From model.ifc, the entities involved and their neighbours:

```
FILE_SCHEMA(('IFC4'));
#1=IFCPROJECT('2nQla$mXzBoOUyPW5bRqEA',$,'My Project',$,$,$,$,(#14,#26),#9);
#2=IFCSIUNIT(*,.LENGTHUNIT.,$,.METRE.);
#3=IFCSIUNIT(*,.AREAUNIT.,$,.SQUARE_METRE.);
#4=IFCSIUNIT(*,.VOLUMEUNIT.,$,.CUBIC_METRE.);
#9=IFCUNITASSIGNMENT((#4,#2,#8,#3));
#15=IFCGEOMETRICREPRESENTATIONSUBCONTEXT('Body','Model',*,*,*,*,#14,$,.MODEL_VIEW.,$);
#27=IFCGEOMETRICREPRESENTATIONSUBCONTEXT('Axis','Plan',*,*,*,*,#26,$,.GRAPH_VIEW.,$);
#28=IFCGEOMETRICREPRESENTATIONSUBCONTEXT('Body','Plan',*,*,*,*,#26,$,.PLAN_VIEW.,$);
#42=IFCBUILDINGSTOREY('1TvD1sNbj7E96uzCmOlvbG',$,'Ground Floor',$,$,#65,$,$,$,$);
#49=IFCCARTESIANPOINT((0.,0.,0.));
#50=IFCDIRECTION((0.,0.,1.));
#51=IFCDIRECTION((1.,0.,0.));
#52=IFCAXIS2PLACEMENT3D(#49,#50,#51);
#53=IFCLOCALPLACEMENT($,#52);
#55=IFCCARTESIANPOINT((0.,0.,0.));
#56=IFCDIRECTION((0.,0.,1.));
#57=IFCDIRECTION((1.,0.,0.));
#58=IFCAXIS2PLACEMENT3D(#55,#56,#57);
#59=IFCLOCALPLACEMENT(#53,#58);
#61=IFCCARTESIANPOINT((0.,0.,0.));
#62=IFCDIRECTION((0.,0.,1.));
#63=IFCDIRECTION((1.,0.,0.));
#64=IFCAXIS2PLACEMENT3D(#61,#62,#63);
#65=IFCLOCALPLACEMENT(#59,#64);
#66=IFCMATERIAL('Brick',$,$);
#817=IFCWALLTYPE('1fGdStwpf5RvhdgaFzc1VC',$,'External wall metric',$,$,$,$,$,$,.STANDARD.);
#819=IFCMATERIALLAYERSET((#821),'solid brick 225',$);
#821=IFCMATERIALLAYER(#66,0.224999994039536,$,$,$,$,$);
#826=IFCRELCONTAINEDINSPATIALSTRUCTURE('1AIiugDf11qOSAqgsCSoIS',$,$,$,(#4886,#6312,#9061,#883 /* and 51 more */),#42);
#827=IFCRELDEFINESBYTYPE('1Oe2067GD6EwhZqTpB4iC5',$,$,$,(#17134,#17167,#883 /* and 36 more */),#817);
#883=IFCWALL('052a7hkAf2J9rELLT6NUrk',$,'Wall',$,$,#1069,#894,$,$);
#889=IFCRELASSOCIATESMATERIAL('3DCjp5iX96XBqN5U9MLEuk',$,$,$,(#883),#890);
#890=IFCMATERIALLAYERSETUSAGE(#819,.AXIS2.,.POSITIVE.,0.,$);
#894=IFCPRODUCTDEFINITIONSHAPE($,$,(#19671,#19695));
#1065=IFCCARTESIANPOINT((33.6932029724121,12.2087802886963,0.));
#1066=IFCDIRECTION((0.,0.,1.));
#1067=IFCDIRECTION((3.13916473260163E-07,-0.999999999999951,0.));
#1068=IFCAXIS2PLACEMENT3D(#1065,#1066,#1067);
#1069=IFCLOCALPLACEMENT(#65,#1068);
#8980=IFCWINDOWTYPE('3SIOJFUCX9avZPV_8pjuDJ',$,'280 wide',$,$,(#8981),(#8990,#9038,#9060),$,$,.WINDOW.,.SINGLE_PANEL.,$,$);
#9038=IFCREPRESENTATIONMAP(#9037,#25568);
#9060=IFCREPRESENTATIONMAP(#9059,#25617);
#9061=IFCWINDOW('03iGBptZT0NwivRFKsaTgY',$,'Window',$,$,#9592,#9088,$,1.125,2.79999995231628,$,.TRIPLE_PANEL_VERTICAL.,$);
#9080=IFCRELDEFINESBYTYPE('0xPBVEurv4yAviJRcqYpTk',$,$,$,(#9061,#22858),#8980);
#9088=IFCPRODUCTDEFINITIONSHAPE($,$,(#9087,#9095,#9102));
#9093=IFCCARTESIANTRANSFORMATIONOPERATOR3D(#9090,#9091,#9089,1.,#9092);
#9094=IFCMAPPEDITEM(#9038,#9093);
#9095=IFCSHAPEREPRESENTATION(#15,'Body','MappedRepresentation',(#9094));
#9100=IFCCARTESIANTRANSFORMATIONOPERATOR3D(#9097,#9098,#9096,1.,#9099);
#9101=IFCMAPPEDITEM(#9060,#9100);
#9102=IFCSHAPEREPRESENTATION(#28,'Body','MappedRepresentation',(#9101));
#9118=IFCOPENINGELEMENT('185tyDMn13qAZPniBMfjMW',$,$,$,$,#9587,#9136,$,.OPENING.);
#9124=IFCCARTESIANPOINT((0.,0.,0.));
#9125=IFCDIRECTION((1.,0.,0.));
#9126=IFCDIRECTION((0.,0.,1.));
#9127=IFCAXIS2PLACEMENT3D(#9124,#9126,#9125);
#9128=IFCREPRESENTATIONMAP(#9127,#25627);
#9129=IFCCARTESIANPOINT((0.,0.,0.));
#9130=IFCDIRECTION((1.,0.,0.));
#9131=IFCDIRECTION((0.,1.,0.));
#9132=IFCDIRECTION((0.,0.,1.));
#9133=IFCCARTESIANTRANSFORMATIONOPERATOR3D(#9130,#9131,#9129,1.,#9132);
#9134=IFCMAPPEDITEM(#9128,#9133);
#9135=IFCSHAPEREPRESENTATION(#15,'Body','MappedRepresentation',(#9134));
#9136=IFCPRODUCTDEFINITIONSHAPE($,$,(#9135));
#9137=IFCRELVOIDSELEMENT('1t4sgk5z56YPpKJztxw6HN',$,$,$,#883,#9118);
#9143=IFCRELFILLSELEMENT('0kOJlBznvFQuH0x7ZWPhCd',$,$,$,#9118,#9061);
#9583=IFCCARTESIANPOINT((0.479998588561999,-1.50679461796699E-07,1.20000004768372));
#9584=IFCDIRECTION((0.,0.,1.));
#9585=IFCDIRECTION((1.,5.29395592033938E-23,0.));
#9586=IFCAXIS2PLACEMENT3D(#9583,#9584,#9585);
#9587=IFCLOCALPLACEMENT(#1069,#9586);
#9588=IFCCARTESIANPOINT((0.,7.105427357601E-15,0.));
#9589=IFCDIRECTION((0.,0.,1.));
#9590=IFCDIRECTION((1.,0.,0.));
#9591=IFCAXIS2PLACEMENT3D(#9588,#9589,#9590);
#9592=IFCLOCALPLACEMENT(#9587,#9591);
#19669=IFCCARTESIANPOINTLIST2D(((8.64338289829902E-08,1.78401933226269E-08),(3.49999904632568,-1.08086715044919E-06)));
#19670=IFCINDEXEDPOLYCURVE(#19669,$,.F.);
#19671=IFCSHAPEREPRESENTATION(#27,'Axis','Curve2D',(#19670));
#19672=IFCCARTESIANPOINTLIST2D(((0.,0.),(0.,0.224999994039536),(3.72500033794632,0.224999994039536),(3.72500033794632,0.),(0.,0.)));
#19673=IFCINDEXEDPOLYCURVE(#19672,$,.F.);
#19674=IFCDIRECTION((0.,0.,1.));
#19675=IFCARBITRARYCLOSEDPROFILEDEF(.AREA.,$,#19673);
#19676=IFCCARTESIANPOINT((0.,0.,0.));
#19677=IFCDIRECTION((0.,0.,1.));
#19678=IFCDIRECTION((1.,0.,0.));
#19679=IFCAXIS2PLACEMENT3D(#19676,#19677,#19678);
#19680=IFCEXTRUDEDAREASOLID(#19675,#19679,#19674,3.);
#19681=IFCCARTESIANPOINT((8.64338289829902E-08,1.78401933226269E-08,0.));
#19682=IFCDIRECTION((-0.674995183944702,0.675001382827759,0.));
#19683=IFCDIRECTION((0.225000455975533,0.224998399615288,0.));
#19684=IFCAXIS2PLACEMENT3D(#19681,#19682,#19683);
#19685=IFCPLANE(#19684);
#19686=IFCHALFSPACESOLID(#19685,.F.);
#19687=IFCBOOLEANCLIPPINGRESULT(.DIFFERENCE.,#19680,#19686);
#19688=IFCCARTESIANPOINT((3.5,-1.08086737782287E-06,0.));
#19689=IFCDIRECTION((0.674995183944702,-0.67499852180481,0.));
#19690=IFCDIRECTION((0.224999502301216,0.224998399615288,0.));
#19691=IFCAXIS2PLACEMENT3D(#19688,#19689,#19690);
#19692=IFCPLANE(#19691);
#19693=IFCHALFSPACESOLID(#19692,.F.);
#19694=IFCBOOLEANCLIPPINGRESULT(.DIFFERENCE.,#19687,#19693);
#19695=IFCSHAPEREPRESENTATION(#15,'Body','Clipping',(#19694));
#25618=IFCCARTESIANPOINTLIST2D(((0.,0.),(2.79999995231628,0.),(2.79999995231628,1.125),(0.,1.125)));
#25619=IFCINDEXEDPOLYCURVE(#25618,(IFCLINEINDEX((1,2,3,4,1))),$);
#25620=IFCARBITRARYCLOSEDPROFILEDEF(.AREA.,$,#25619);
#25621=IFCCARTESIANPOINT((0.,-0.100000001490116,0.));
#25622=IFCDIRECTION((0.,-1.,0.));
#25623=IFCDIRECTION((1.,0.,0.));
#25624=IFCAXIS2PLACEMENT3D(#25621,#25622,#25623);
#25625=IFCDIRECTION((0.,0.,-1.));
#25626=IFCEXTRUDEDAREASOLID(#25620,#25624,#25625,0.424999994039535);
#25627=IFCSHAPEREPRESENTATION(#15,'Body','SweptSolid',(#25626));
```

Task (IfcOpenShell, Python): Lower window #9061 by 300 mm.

```python
import numpy as np
import ifcopenshell
import ifcopenshell.api.geometry
import ifcopenshell.util.placement
import ifcopenshell.util.unit

model = ifcopenshell.open("model.ifc")
unit_scale = ifcopenshell.util.unit.calculate_unit_scale(model)

window = model.by_guid("03iGBptZT0NwivRFKsaTgY")
opening = window.FillsVoids[0].RelatingOpeningElement
dz = -0.3

shift = np.array([0.0, 0.0, dz])
# The window is placed relative to its opening, so it follows when the opening moves.
matrix = ifcopenshell.util.placement.get_local_placement(opening.ObjectPlacement)
matrix[:3, 3] += shift
ifcopenshell.api.geometry.edit_object_placement(
    model, product=opening, matrix=matrix, is_si=False, should_transform_children=True
)

print(f"moved by {dz * unit_scale:+.3f} m")

model.write("model_v2.ifc")
```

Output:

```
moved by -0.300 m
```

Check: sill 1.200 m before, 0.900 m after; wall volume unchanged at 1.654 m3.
